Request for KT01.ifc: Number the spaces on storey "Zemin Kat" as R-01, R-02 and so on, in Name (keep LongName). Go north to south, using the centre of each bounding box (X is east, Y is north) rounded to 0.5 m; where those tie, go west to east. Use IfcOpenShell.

First a look at what the model holds.

```python
import ifcopenshell
import ifcopenshell.util.element
import ifcopenshell.util.placement

model = ifcopenshell.open("KT01.ifc")
print(model.schema)
storey = next(s for s in model.by_type("IfcBuildingStorey") if s.Name == "Zemin Kat")
spaces = [e for e in ifcopenshell.util.element.get_decomposition(storey) if e.is_a("IfcSpace")]
for e in sorted(spaces, key=lambda e: e.id()):
    origin = ifcopenshell.util.placement.get_local_placement(e.ObjectPlacement)[:3, 3]
    print(e.id(), e.Name, e.LongName, origin.round(2) + 0.0, sep=" | ")
```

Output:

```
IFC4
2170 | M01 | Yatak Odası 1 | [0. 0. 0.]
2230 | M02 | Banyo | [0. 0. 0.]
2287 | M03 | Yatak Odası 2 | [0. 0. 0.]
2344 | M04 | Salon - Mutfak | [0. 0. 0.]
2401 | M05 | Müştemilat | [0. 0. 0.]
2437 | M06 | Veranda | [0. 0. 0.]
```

```python
import ifcopenshell
import ifcopenshell.geom
import ifcopenshell.util.element
import ifcopenshell.util.shape

model = ifcopenshell.open("KT01.ifc")
settings = ifcopenshell.geom.settings()
settings.set("use-world-coords", True)


def centre(element):
    shape = ifcopenshell.geom.create_shape(settings, element)
    return ifcopenshell.util.shape.get_bbox_centroid(shape.geometry)


storey = next(s for s in model.by_type("IfcBuildingStorey") if s.Name == "Zemin Kat")
spaces = [e for e in ifcopenshell.util.element.get_decomposition(storey) if e.is_a("IfcSpace")]

# Insertion points can sit at a corner or the storey origin, so sort by the geometry (in metres).
centres = {e: centre(e) for e in spaces}
spaces.sort(key=lambda e: (-round(centres[e][1] / 0.5), centres[e][0]))

for i, e in enumerate(spaces, start=1):
    number = f"R-{i:02d}"
    e.Name = number
    print(e.id(), number)

model.write("KT01_v2.ifc")
```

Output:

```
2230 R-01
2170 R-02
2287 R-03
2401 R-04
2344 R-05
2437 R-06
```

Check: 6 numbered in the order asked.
